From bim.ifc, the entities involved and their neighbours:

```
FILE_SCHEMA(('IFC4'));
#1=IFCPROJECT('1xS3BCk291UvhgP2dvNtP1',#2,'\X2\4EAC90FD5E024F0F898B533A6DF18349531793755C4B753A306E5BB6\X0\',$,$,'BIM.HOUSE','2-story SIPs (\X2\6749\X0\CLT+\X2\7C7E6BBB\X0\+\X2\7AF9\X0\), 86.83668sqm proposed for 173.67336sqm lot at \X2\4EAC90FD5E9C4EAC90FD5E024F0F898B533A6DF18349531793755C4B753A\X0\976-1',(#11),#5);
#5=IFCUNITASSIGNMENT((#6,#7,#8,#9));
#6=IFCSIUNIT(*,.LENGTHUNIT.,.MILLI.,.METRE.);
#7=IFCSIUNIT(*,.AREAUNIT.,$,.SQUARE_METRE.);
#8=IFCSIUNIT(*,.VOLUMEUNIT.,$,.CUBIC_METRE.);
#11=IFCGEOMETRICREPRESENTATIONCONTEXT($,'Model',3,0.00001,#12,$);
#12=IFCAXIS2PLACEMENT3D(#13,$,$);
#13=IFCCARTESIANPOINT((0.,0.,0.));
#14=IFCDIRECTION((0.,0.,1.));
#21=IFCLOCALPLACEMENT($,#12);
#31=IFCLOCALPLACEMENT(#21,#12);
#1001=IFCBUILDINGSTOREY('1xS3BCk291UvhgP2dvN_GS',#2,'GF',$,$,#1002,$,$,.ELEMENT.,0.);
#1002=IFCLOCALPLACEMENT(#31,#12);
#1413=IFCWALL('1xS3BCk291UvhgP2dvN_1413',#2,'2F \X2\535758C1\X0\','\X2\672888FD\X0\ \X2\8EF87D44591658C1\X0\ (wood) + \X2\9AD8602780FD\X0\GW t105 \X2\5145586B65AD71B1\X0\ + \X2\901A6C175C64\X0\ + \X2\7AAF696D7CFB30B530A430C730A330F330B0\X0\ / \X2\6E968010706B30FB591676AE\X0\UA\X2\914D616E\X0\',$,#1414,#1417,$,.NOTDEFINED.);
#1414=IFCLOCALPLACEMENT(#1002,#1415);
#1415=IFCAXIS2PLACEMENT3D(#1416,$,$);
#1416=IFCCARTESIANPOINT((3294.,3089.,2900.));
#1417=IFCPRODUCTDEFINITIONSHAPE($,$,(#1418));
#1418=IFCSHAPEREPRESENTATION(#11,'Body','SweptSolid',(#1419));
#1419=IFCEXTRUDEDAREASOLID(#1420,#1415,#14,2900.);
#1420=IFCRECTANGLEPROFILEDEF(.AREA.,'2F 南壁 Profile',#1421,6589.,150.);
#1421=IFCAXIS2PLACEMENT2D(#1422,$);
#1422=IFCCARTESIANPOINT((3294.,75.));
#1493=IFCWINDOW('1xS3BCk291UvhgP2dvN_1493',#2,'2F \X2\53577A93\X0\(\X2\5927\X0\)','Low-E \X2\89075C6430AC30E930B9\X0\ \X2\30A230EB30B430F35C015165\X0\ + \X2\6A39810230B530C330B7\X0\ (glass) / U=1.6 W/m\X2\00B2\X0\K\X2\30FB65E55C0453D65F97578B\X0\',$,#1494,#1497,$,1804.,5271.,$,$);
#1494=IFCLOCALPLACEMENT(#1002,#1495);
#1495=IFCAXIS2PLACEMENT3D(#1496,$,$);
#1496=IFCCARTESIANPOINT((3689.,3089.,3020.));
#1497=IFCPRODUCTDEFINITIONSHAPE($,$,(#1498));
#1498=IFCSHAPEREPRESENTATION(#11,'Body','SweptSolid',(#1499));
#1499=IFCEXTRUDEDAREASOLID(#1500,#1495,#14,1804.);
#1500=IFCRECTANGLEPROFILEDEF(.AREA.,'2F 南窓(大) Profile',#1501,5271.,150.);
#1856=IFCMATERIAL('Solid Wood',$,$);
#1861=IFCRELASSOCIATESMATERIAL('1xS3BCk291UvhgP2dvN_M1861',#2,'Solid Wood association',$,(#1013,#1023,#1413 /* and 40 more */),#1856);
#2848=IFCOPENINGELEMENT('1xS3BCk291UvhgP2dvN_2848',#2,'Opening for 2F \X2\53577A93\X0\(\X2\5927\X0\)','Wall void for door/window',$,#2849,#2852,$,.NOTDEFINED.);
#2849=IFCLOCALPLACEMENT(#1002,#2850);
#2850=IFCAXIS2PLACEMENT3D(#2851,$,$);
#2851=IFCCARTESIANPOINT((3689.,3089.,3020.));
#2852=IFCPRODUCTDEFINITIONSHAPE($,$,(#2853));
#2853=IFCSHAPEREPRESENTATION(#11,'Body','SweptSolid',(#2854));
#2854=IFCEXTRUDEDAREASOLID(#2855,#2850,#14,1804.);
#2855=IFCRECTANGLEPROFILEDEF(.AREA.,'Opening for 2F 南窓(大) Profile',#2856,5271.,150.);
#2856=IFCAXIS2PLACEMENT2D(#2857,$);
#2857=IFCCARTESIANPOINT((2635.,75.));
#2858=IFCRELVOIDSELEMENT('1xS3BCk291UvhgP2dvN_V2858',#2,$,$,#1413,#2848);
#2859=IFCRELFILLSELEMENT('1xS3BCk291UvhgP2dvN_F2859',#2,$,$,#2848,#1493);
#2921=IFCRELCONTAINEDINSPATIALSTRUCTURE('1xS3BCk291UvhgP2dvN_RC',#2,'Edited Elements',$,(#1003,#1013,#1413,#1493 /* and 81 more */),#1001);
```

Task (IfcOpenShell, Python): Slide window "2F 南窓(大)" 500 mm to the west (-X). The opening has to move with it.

```python
import ifcopenshell
import ifcopenshell.api.geometry
import ifcopenshell.util.placement

model = ifcopenshell.open("bim.ifc")

window = model.by_id(1493)
opening = window.FillsVoids[0].RelatingOpeningElement
wall = opening.VoidsElements[0].RelatingBuildingElement

wall_matrix = ifcopenshell.util.placement.get_local_placement(wall.ObjectPlacement)
shift = wall_matrix[:3, 0] * -500.0
before = ifcopenshell.util.placement.get_local_placement(window.ObjectPlacement)[:3, 3].copy()

# The window is not placed relative to its opening, so move both.
for product in (opening, window):
    matrix = ifcopenshell.util.placement.get_local_placement(product.ObjectPlacement)
    matrix[:3, 3] += shift
    ifcopenshell.api.geometry.edit_object_placement(model, product=product, matrix=matrix, is_si=False)

after = ifcopenshell.util.placement.get_local_placement(window.ObjectPlacement)[:3, 3]
print("window moved by", (after - before).round(3) + 0.0)

model.write("bim_rev.ifc")
```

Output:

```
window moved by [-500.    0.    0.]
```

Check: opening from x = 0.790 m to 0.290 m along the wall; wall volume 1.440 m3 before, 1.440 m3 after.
